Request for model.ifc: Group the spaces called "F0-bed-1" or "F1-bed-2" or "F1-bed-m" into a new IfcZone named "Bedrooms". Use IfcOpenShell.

First a look at what the model holds.

```python
import ifcopenshell

model = ifcopenshell.open("model.ifc")
print(model.schema)
seen = {}
for space in model.by_type("IfcSpace"):
    seen[space.LongName] = seen.get(space.LongName, 0) + 1
for name, count in sorted(seen.items(), key=str):
    print(count, "x", name)
print("zones:", [z.Name for z in model.by_type("IfcZone")][:20])
```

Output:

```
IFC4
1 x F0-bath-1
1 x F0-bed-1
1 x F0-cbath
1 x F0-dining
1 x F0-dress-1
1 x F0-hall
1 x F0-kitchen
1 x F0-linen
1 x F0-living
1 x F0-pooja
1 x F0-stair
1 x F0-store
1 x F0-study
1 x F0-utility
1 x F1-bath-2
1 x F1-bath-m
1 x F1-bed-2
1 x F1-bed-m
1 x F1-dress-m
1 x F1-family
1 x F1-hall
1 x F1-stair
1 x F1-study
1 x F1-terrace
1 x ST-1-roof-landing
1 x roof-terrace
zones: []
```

```python
import ifcopenshell
import ifcopenshell.api.group
import ifcopenshell.api.root

model = ifcopenshell.open("model.ifc")

names = {"F0-bed-1", "F1-bed-2", "F1-bed-m"}
spaces = [s for s in model.by_type("IfcSpace") if s.LongName in names]

zone = ifcopenshell.api.root.create_entity(model, ifc_class="IfcZone", name="Bedrooms")
ifcopenshell.api.group.assign_group(model, products=spaces, group=zone)
print(len(spaces), "spaces in", zone.Name)

model.write("model_v2.ifc")
```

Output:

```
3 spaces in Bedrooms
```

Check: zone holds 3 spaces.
